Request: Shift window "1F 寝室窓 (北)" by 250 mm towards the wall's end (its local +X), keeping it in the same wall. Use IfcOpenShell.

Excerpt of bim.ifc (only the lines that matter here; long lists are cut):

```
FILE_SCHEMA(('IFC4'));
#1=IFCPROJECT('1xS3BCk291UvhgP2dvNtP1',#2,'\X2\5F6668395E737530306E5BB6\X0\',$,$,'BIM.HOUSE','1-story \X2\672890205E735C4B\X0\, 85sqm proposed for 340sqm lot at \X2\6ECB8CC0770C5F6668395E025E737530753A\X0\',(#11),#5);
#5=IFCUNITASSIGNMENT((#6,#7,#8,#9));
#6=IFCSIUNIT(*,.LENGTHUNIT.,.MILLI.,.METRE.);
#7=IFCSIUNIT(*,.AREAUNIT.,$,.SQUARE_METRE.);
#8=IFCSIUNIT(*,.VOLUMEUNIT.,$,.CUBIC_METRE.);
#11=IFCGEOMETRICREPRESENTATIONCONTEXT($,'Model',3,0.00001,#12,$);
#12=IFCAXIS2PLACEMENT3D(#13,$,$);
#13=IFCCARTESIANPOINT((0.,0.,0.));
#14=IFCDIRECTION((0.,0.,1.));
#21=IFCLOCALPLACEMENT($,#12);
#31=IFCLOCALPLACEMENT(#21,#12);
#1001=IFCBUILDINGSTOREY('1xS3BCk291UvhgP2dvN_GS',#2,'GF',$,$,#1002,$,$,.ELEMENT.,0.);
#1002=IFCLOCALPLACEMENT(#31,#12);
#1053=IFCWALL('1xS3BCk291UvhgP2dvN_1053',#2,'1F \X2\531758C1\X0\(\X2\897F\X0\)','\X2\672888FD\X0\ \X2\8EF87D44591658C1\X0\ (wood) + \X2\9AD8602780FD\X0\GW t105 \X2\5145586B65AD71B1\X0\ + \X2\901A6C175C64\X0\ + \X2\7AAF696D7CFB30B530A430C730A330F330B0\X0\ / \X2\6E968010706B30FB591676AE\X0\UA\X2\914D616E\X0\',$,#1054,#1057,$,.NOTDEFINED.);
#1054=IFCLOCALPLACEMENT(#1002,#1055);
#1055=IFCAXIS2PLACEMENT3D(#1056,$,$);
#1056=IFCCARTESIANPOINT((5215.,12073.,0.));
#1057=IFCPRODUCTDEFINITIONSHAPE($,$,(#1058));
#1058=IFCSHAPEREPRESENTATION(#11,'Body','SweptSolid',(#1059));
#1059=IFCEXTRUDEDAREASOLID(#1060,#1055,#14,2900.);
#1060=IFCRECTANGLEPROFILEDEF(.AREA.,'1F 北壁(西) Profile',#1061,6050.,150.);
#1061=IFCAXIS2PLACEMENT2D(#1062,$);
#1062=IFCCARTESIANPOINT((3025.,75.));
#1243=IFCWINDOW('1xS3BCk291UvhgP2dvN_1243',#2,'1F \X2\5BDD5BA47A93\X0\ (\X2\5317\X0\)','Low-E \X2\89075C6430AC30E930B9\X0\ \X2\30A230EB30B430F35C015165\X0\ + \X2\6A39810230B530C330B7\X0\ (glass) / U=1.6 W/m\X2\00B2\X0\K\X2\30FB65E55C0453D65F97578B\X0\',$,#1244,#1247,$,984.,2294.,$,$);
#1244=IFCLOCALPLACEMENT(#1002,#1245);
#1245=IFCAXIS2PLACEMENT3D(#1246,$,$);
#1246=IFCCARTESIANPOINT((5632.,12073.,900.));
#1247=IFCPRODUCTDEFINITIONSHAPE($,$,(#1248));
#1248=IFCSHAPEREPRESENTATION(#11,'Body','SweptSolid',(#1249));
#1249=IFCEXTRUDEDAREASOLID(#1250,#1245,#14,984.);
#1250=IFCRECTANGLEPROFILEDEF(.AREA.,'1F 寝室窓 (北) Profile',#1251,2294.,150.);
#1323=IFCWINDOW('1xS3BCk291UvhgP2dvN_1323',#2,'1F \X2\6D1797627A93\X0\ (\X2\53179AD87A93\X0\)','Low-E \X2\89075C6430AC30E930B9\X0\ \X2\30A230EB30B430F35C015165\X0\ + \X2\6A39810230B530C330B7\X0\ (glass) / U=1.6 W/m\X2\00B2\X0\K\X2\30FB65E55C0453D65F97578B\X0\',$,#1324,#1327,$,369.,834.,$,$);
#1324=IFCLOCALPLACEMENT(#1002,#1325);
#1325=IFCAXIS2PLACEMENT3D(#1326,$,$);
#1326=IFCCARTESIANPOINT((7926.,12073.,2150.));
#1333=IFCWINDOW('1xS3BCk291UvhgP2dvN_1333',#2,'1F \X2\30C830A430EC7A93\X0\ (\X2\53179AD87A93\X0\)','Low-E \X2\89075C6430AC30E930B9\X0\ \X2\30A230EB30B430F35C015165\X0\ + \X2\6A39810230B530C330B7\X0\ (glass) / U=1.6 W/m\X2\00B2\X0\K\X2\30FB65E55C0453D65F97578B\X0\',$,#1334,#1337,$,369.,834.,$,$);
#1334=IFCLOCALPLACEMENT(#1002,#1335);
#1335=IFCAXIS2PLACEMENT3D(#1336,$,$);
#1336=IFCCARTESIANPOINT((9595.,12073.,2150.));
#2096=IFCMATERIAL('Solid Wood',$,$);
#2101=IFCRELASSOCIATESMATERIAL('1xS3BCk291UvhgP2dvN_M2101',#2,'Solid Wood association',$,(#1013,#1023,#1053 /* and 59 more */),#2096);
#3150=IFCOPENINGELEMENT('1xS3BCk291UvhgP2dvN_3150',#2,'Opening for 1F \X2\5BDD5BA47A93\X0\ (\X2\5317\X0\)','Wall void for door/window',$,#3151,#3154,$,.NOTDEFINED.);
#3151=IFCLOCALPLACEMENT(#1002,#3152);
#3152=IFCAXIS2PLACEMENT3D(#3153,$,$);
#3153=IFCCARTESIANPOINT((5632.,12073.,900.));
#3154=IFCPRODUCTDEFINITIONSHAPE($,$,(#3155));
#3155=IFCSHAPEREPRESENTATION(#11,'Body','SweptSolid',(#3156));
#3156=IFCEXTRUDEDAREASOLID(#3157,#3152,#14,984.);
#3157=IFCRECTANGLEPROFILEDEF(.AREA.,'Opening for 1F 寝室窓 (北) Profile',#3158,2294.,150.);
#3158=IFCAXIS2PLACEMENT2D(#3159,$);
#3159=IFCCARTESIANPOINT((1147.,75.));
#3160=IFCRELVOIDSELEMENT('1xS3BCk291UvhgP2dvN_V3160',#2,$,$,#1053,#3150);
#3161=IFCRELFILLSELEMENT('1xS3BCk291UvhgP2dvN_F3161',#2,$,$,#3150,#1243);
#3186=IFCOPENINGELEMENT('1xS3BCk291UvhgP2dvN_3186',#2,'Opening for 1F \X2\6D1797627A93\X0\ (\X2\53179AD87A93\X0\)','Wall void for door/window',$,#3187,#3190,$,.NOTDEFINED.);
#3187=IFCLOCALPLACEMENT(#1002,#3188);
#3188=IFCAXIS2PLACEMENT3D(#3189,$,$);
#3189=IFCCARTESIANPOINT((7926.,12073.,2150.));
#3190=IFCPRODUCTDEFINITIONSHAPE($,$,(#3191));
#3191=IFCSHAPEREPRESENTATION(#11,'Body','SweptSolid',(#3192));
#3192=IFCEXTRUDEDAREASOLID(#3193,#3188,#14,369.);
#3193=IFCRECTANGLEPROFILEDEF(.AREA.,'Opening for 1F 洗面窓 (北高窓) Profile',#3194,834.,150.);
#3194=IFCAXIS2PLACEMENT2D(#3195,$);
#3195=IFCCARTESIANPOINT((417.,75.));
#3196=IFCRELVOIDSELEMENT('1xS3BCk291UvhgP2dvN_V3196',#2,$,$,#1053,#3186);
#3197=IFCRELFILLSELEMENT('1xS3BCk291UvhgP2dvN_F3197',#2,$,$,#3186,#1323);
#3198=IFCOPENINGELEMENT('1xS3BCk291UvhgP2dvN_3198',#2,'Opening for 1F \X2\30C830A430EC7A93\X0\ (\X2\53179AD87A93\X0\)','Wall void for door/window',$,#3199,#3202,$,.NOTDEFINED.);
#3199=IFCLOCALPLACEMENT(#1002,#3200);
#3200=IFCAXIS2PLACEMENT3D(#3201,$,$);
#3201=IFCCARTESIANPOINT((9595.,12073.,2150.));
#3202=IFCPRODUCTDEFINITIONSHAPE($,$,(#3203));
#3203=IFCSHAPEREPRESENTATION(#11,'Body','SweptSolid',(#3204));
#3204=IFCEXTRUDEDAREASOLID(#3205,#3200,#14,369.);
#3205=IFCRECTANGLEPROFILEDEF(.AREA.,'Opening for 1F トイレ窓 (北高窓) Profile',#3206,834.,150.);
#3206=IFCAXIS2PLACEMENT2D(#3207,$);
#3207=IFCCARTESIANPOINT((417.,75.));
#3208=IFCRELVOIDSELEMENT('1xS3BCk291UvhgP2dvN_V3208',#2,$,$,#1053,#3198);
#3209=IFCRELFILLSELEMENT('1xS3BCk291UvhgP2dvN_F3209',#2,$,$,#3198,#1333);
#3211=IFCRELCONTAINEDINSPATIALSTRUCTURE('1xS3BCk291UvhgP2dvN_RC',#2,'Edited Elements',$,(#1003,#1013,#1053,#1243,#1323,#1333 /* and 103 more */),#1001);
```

```python
import ifcopenshell
import ifcopenshell.api.geometry
import ifcopenshell.util.placement

model = ifcopenshell.open("bim.ifc")

window = model.by_guid("1xS3BCk291UvhgP2dvN_1243")
opening = window.FillsVoids[0].RelatingOpeningElement
wall = opening.VoidsElements[0].RelatingBuildingElement

wall_matrix = ifcopenshell.util.placement.get_local_placement(wall.ObjectPlacement)
shift = wall_matrix[:3, 0] * 250.0
before = ifcopenshell.util.placement.get_local_placement(window.ObjectPlacement)[:3, 3].copy()

# The window is not placed relative to its opening, so move both.
for product in (opening, window):
    matrix = ifcopenshell.util.placement.get_local_placement(product.ObjectPlacement)
    matrix[:3, 3] += shift
    ifcopenshell.api.geometry.edit_object_placement(model, product=product, matrix=matrix, is_si=False)

after = ifcopenshell.util.placement.get_local_placement(window.ObjectPlacement)[:3, 3]
print("window moved by", (after - before).round(3) + 0.0)

model.write("bim_edited.ifc")
```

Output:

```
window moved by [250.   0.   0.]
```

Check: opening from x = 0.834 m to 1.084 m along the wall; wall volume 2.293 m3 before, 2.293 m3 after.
